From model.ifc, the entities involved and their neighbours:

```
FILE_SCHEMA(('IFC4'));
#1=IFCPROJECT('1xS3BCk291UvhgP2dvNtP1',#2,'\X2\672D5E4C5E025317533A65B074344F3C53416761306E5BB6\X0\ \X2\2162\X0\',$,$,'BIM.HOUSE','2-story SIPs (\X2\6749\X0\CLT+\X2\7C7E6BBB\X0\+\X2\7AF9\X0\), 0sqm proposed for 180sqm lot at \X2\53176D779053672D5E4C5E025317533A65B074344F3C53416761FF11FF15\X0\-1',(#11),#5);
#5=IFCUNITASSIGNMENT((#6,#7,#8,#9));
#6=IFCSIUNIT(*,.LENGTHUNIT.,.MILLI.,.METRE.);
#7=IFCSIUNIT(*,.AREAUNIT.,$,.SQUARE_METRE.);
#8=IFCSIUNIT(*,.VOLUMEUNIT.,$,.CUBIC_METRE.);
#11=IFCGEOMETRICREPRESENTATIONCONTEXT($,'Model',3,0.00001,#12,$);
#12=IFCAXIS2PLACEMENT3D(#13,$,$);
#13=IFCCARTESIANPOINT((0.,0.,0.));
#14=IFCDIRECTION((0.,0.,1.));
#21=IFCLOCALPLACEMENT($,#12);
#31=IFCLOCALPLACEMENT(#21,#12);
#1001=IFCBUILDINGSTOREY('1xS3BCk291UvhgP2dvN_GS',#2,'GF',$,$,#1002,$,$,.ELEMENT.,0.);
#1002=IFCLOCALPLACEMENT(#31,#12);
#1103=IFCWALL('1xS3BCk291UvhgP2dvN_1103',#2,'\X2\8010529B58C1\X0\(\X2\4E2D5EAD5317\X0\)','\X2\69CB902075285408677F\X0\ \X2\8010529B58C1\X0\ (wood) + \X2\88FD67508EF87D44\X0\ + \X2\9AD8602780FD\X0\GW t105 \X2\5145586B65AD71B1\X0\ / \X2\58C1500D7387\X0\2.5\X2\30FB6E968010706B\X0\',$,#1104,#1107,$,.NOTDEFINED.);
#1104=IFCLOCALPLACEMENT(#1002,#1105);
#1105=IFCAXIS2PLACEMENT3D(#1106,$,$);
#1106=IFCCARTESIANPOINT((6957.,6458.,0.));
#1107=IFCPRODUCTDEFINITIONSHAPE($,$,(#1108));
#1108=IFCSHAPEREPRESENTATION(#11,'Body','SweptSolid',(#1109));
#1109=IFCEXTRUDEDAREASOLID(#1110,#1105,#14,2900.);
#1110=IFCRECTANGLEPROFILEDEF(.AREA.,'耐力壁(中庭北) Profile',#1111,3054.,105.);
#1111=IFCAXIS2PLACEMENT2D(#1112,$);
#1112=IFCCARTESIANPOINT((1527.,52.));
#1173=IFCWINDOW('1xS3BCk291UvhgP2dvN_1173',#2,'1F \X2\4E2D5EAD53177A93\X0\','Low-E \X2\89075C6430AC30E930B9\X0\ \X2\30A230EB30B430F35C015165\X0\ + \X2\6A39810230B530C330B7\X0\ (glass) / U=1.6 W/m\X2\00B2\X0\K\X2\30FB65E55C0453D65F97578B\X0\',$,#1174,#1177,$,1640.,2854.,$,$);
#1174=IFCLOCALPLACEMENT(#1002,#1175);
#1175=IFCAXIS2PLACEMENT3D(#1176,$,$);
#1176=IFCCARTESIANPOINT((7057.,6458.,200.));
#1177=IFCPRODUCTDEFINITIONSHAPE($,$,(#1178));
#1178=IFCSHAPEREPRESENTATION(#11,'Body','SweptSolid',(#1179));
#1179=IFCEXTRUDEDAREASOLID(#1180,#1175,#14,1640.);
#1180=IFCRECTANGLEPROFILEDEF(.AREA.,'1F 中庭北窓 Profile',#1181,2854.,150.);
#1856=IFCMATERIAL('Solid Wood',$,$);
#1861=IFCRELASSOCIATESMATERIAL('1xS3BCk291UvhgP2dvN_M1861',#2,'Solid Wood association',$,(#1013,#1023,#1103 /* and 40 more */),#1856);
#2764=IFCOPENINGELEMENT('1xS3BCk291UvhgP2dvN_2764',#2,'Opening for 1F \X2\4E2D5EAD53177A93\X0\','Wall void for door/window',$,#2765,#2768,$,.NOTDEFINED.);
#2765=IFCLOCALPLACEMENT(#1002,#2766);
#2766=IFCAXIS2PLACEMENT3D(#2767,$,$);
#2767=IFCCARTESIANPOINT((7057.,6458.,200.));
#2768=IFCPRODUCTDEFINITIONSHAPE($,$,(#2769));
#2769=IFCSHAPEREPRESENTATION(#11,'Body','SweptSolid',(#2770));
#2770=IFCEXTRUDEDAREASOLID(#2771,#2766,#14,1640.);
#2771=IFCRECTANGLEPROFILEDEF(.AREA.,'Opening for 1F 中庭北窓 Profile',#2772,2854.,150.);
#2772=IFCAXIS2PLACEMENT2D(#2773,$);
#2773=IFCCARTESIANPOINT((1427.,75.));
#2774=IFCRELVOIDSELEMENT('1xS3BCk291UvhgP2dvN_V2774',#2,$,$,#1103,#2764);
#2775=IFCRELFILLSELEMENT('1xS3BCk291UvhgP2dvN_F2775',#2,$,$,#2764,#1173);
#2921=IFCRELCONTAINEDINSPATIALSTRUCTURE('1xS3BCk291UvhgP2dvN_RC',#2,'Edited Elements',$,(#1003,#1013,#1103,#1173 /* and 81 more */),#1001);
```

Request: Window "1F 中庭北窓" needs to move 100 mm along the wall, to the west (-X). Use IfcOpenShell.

```python
import ifcopenshell
import ifcopenshell.api.geometry
import ifcopenshell.util.placement

model = ifcopenshell.open("model.ifc")

window = model.by_guid("1xS3BCk291UvhgP2dvN_1173")
opening = window.FillsVoids[0].RelatingOpeningElement
wall = opening.VoidsElements[0].RelatingBuildingElement

wall_matrix = ifcopenshell.util.placement.get_local_placement(wall.ObjectPlacement)
shift = wall_matrix[:3, 0] * -100.0
before = ifcopenshell.util.placement.get_local_placement(window.ObjectPlacement)[:3, 3].copy()

# The window is not placed relative to its opening, so move both.
for product in (opening, window):
    matrix = ifcopenshell.util.placement.get_local_placement(product.ObjectPlacement)
    matrix[:3, 3] += shift
    ifcopenshell.api.geometry.edit_object_placement(model, product=product, matrix=matrix, is_si=False)

after = ifcopenshell.util.placement.get_local_placement(window.ObjectPlacement)[:3, 3]
print("window moved by", (after - before).round(3) + 0.0)

model.write("model_updated.ifc")
```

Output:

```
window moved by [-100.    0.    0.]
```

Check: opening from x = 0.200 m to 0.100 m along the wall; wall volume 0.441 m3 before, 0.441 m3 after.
